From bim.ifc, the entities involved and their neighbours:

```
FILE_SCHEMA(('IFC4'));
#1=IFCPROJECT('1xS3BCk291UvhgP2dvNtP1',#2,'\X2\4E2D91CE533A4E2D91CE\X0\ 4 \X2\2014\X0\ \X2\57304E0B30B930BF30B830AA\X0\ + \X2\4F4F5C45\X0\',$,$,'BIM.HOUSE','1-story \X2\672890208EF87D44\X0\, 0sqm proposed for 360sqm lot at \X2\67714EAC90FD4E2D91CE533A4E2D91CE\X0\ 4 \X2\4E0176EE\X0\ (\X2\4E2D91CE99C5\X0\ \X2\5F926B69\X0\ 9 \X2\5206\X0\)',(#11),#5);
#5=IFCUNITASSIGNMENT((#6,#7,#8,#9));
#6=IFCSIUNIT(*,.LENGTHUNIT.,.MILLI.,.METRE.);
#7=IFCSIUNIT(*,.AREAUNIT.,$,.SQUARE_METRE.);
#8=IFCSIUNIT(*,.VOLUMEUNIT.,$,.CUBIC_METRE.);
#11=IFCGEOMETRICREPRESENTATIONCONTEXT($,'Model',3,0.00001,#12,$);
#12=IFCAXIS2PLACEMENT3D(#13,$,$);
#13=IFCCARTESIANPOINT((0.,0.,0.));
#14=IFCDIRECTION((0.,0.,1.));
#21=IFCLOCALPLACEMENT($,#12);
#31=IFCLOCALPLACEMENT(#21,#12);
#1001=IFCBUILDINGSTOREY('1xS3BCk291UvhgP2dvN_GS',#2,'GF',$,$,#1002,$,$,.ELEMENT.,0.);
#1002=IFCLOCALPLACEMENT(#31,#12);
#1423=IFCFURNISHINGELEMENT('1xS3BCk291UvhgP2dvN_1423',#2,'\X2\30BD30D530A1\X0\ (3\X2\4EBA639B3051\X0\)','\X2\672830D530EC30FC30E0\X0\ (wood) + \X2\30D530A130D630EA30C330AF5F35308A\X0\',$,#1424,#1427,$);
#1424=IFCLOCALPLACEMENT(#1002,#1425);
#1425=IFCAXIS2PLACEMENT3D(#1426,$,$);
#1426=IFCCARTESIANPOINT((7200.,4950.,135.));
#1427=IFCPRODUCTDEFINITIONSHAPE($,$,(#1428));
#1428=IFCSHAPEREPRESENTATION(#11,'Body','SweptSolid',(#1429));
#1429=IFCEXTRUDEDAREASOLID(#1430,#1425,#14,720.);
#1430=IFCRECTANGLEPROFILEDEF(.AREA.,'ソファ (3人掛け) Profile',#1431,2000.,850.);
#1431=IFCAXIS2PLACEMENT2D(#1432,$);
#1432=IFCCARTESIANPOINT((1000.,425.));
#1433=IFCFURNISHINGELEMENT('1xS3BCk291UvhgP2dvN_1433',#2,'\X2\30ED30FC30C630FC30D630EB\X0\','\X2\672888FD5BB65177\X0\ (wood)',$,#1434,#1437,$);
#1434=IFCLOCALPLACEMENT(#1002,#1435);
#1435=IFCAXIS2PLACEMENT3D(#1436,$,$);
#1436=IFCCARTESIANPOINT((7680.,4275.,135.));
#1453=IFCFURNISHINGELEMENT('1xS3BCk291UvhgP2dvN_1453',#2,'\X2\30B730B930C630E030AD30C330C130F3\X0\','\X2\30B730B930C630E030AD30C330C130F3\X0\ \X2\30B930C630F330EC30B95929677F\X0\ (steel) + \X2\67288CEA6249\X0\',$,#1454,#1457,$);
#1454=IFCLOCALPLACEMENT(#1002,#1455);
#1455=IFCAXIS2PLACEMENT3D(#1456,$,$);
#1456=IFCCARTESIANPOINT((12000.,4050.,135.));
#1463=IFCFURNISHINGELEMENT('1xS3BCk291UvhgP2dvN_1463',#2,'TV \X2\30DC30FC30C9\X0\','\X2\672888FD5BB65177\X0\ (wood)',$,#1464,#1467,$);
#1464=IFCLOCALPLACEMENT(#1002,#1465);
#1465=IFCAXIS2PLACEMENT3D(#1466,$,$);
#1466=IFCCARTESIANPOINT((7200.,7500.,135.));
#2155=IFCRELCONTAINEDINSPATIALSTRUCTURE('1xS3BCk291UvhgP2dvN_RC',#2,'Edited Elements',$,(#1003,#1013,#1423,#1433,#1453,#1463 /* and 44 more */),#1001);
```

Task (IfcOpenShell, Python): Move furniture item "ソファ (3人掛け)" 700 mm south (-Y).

```python
import ifcopenshell
import ifcopenshell.api.geometry
import ifcopenshell.util.placement
import ifcopenshell.util.unit

model = ifcopenshell.open("bim.ifc")
unit_scale = ifcopenshell.util.unit.calculate_unit_scale(model)

item = model.by_id(1423)
matrix = ifcopenshell.util.placement.get_local_placement(item.ObjectPlacement)
matrix[1, 3] -= 0.7 / unit_scale
ifcopenshell.api.geometry.edit_object_placement(model, product=item, matrix=matrix, is_si=False)

print(ifcopenshell.util.placement.get_local_placement(item.ObjectPlacement).round(3) + 0.0)

model.write("bim_v2.ifc")
```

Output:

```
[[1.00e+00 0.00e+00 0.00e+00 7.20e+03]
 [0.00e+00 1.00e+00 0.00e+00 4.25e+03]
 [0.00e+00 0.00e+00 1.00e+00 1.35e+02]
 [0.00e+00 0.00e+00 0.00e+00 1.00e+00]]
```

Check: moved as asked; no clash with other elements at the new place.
